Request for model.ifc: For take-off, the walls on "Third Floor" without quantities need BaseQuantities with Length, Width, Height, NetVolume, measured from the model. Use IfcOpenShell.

First a look at what the model holds.

```python
import ifcopenshell
import ifcopenshell.util.element
import ifcopenshell.util.unit

model = ifcopenshell.open("model.ifc")
print(model.schema)
for unit_type in ("LENGTHUNIT", "AREAUNIT", "VOLUMEUNIT"):
    print(unit_type, ifcopenshell.util.unit.calculate_unit_scale(model, unit_type))
storey = next(s for s in model.by_type("IfcBuildingStorey") if s.Name == "Third Floor")
walls = [e for e in ifcopenshell.util.element.get_decomposition(storey) if e.is_a("IfcWall")]
for e in sorted(walls, key=lambda e: e.id()):
    print(e.id(), e.is_a(), e.Name, list(ifcopenshell.util.element.get_psets(e, qtos_only=True)), sep=" | ")
```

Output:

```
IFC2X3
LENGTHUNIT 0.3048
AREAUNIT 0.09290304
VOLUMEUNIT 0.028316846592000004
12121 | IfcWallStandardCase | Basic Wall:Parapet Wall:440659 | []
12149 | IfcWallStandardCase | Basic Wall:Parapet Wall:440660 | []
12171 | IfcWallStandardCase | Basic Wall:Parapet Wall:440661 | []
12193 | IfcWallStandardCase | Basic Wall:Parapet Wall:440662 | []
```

```python
import ifcopenshell
import ifcopenshell.api.pset
import ifcopenshell.geom
import ifcopenshell.util.element
import ifcopenshell.util.shape
import ifcopenshell.util.unit

model = ifcopenshell.open("model.ifc")
unit_scale = ifcopenshell.util.unit.calculate_unit_scale(model)
volume_scale = ifcopenshell.util.unit.calculate_unit_scale(model, "VOLUMEUNIT")
settings = ifcopenshell.geom.settings()

storey = next(s for s in model.by_type("IfcBuildingStorey") if s.Name == "Third Floor")
walls = [e for e in ifcopenshell.util.element.get_decomposition(storey) if e.is_a("IfcWall")]

for e in sorted(walls, key=lambda e: e.id()):
    if ifcopenshell.util.element.get_psets(e, qtos_only=True, should_inherit=False):
        continue
    # Geometry comes back in metres, in the element's own axes.
    shape = ifcopenshell.geom.create_shape(settings, e)
    values = {
        "Length": ifcopenshell.util.shape.get_x(shape.geometry) / unit_scale,
        "Width": ifcopenshell.util.shape.get_y(shape.geometry) / unit_scale,
        "Height": ifcopenshell.util.shape.get_z(shape.geometry) / unit_scale,
        "NetVolume": ifcopenshell.util.shape.get_volume(shape.geometry) / volume_scale,
    }
    qto = ifcopenshell.api.pset.add_qto(model, product=e, name="BaseQuantities")
    ifcopenshell.api.pset.edit_qto(model, qto=qto, properties=values)
    print(e.id(), {k: round(v, 3) for k, v in values.items()})

model.write("model_rev.ifc")
```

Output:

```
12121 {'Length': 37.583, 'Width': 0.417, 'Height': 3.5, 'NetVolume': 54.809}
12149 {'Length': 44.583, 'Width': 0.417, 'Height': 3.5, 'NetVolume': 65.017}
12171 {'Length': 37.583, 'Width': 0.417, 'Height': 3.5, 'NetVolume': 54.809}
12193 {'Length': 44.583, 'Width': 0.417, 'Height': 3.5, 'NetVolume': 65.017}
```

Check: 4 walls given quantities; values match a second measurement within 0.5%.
